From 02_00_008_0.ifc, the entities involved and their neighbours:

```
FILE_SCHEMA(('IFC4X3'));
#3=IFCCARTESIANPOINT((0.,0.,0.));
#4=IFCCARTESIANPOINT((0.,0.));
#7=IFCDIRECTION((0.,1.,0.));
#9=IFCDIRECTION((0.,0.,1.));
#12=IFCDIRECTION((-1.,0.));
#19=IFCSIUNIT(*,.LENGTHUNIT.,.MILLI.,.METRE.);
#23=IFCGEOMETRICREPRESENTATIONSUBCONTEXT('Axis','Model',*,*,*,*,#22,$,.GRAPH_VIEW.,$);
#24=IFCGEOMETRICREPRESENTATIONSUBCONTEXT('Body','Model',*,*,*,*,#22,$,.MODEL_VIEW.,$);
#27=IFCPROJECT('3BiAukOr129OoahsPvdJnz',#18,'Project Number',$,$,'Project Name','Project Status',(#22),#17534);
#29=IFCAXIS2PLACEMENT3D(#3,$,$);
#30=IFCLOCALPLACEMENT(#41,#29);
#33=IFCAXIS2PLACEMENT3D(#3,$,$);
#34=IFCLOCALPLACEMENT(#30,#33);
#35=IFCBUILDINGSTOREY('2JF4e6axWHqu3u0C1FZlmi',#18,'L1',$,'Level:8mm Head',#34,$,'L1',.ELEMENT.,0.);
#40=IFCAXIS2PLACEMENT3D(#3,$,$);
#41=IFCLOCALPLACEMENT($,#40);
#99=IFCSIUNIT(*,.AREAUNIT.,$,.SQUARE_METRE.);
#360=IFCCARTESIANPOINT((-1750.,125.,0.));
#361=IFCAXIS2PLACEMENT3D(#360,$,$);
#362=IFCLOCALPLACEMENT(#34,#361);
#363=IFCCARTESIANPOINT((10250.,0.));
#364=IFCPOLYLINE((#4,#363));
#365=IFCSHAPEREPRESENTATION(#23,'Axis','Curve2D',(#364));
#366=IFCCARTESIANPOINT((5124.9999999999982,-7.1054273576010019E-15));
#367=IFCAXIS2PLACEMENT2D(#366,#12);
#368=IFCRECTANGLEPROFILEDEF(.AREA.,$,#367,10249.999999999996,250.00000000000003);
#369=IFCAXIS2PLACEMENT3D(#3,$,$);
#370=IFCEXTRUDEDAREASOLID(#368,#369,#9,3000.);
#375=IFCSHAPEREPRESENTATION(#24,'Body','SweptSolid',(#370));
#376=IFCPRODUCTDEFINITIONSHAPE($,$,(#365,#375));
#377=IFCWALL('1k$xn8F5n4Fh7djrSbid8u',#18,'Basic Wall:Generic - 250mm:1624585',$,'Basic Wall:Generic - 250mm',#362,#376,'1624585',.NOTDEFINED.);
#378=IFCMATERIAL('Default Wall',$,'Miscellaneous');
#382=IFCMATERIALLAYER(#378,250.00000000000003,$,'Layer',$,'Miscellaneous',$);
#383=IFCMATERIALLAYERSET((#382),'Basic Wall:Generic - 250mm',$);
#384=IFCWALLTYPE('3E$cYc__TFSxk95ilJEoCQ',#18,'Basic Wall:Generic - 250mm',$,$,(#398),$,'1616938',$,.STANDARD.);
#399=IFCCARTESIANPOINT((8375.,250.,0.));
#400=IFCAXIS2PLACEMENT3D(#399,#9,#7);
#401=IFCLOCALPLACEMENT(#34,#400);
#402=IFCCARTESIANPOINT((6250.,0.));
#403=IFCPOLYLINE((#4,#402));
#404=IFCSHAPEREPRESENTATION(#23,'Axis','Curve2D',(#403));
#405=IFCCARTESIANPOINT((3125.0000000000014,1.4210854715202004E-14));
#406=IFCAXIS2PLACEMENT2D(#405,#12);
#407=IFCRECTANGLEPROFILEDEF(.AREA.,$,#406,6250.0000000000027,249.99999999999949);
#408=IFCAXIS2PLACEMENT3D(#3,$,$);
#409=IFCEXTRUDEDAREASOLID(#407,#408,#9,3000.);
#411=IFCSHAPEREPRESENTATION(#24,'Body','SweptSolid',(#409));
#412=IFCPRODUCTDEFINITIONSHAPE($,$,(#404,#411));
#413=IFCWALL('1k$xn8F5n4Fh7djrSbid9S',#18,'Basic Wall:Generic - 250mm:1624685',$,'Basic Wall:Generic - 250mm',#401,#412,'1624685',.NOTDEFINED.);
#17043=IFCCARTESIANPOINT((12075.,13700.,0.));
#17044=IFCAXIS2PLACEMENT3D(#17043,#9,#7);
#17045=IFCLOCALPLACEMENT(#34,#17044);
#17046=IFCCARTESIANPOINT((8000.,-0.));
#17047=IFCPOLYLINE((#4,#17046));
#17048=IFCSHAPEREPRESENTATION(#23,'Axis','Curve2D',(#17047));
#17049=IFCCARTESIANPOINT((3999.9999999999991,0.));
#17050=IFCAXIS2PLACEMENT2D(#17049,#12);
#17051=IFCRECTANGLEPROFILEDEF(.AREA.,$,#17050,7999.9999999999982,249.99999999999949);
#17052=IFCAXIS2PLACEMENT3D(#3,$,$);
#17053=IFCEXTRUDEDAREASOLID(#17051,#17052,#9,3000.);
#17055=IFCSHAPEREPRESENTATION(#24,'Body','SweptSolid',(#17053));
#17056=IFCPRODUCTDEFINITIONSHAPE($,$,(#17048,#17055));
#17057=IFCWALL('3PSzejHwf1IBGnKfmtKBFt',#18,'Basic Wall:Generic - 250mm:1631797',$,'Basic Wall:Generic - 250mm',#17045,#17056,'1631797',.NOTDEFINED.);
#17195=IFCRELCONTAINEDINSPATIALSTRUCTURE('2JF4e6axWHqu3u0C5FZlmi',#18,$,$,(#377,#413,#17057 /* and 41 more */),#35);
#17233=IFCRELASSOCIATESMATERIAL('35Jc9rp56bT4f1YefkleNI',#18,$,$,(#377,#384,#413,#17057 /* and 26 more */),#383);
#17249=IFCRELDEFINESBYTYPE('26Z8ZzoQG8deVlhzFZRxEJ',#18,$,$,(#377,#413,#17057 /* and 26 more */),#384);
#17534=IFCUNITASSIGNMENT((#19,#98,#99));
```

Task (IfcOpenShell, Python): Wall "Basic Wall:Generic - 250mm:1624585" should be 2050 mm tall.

```python
import ifcopenshell
import ifcopenshell.geom
import ifcopenshell.util.representation
import ifcopenshell.util.shape

model = ifcopenshell.open("02_00_008_0.ifc")
settings = ifcopenshell.geom.settings()


def volume(element):
    """Net volume in cubic metres, openings subtracted."""
    shape = ifcopenshell.geom.create_shape(settings, element)
    return ifcopenshell.util.shape.get_volume(shape.geometry)


wall = model.by_guid("1k$xn8F5n4Fh7djrSbid8u")
before = volume(wall)

body = ifcopenshell.util.representation.get_representation(wall, "Model", "Body")
solid = body.Items[0]
old_height = solid.Depth
solid.Depth = 2050.0
after = volume(wall)

print(f"height {old_height:g} -> {solid.Depth:g}, volume {before:.3f} -> {after:.3f} m3")

model.write("02_00_008_0_v2.ifc")
```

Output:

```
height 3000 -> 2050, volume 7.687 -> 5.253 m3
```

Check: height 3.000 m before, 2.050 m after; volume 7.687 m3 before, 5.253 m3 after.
